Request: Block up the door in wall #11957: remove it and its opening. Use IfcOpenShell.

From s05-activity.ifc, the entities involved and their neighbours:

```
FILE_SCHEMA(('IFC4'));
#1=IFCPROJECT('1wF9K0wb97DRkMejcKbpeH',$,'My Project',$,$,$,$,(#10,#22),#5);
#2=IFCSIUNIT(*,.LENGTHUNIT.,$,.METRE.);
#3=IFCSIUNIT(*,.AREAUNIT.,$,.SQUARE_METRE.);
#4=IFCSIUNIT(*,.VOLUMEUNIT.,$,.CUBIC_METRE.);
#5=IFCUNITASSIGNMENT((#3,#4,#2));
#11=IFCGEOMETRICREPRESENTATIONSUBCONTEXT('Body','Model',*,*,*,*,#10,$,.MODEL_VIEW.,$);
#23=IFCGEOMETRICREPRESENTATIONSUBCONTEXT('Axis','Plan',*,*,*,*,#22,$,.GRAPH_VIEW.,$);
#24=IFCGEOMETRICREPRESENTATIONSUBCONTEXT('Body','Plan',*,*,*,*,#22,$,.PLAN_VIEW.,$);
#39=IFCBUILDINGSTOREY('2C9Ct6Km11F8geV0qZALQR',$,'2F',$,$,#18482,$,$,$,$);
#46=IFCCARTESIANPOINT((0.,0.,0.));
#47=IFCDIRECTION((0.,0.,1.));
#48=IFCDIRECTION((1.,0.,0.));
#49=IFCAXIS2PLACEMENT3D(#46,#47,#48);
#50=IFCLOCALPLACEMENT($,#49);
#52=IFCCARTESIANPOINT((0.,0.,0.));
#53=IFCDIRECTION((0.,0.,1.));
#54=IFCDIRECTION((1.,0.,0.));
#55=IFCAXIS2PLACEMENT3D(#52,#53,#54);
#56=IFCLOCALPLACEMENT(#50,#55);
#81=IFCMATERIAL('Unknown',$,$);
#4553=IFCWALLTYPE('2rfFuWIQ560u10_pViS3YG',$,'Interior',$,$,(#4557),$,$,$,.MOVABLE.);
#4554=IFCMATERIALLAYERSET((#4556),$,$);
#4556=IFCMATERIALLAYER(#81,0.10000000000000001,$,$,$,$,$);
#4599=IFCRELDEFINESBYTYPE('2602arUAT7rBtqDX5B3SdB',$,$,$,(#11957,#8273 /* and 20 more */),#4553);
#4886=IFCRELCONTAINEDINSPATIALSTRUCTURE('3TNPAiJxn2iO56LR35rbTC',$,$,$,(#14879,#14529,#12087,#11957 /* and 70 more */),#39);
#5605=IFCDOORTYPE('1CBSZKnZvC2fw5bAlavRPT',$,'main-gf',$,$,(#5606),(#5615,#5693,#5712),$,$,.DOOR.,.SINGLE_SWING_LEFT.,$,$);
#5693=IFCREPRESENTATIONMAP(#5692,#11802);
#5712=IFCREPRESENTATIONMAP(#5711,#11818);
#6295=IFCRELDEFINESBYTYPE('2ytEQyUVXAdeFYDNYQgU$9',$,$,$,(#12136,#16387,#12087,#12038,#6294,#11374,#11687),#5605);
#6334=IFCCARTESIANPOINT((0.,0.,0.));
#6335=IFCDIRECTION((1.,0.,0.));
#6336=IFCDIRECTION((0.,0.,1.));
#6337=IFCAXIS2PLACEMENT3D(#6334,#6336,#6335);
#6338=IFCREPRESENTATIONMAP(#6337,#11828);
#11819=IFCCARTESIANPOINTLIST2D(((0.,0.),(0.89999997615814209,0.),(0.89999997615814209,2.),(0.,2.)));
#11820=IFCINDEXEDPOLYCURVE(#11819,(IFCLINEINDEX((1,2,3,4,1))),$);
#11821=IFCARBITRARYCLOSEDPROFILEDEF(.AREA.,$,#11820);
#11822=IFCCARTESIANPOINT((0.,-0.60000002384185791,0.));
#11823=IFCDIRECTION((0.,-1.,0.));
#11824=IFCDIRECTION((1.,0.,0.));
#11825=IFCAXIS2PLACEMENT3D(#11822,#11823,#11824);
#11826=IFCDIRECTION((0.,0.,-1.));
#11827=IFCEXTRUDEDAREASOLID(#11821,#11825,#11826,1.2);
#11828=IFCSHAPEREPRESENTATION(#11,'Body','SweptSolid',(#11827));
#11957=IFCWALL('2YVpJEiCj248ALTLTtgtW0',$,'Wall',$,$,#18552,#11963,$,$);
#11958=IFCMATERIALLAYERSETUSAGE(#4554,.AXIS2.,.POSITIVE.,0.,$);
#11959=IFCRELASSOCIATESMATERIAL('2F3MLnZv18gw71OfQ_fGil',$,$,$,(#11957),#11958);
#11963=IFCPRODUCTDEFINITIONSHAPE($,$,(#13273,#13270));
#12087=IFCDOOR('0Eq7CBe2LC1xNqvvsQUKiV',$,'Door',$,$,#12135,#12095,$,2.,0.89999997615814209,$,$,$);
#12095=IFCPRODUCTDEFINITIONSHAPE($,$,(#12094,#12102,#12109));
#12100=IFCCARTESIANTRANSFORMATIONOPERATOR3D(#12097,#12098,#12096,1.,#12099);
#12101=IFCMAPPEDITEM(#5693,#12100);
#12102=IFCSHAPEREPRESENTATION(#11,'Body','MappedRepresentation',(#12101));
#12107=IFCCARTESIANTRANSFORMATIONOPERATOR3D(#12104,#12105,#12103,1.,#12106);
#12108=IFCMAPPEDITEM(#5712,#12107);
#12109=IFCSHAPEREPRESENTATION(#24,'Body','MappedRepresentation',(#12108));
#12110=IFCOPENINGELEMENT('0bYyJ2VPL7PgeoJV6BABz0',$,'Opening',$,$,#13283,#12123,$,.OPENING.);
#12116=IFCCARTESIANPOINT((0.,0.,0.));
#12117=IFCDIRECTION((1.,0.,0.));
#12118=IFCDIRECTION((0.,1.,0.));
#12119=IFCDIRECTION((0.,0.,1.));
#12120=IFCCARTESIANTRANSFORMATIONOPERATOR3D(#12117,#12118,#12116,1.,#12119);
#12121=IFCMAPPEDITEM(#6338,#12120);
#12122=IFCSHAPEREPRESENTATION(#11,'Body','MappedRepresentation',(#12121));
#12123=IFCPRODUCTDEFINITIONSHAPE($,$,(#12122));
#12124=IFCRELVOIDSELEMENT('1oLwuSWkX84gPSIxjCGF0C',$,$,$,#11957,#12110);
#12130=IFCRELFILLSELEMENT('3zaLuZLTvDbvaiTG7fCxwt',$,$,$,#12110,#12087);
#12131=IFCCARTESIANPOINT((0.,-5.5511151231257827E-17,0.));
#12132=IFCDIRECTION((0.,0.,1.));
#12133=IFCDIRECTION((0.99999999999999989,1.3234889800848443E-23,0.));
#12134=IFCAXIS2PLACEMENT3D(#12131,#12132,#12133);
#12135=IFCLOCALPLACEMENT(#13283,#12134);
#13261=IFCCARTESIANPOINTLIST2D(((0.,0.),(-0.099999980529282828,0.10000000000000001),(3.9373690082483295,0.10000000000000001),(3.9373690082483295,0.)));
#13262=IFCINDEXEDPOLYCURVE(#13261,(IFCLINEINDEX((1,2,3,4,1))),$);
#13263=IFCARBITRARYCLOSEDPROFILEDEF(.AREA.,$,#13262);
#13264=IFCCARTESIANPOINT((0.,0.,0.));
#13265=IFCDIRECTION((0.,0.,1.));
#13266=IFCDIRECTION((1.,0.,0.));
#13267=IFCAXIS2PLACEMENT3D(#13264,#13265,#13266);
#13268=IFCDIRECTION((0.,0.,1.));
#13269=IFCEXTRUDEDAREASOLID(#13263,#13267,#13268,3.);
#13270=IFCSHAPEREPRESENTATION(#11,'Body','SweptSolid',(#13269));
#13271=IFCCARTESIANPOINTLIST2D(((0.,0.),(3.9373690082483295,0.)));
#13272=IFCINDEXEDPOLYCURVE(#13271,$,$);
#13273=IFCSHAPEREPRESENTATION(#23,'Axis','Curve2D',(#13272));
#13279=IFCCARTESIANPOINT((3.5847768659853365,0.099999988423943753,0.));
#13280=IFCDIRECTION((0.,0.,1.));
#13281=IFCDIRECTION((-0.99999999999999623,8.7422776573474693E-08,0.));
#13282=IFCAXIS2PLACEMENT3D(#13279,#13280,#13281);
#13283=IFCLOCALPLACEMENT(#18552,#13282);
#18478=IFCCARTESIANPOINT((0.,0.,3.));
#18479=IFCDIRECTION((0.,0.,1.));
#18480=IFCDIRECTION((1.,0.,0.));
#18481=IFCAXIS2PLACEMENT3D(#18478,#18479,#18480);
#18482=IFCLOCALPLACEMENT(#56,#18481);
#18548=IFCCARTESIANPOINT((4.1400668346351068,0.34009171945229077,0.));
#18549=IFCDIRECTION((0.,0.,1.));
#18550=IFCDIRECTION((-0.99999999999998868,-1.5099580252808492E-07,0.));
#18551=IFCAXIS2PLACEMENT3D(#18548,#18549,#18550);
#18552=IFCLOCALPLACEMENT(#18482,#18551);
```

```python
import ifcopenshell
import ifcopenshell.api.feature
import ifcopenshell.api.root
import ifcopenshell.geom
import ifcopenshell.util.shape

model = ifcopenshell.open("s05-activity.ifc")
settings = ifcopenshell.geom.settings()


def volume(element):
    """Net volume in cubic metres, openings subtracted."""
    shape = ifcopenshell.geom.create_shape(settings, element)
    return ifcopenshell.util.shape.get_volume(shape.geometry)


door = model.by_guid("0Eq7CBe2LC1xNqvvsQUKiV")
opening = door.FillsVoids[0].RelatingOpeningElement
wall = opening.VoidsElements[0].RelatingBuildingElement
before = volume(wall)

ifcopenshell.api.root.remove_product(model, product=door)
ifcopenshell.api.feature.remove_feature(model, feature=opening)

after = volume(wall)

print(f"wall volume {before:.3f} -> {after:.3f} m3")

model.write("s05-activity_v2.ifc")
```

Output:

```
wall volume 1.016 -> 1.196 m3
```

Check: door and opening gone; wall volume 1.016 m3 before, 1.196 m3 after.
